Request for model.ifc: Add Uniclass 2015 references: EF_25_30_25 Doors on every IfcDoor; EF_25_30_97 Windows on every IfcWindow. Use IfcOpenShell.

First a look at what the model holds.

```python
import ifcopenshell

model = ifcopenshell.open("model.ifc")
print(model.schema)
print("classifications:", [c.Name for c in model.by_type("IfcClassification")])
for ifc_class in ("IfcDoor", "IfcRoof", "IfcStair", "IfcWall", "IfcWindow"):
    print(ifc_class, len(model.by_type(ifc_class)))
```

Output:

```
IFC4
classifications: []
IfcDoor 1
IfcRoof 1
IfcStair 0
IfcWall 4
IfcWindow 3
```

```python
import ifcopenshell
import ifcopenshell.api.classification

model = ifcopenshell.open("model.ifc")

system = ifcopenshell.api.classification.add_classification(model, classification="Uniclass 2015")

codes = {
    "IfcDoor": ("EF_25_30_25", "Doors"),
    "IfcWindow": ("EF_25_30_97", "Windows"),
}
for ifc_class, (code, name) in codes.items():
    products = model.by_type(ifc_class)
    ifcopenshell.api.classification.add_reference(
        model, products=products, classification=system, identification=code, name=name
    )
    print(code, len(products))

model.write("model-out.ifc")
```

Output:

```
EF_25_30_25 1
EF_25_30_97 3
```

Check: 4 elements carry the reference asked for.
